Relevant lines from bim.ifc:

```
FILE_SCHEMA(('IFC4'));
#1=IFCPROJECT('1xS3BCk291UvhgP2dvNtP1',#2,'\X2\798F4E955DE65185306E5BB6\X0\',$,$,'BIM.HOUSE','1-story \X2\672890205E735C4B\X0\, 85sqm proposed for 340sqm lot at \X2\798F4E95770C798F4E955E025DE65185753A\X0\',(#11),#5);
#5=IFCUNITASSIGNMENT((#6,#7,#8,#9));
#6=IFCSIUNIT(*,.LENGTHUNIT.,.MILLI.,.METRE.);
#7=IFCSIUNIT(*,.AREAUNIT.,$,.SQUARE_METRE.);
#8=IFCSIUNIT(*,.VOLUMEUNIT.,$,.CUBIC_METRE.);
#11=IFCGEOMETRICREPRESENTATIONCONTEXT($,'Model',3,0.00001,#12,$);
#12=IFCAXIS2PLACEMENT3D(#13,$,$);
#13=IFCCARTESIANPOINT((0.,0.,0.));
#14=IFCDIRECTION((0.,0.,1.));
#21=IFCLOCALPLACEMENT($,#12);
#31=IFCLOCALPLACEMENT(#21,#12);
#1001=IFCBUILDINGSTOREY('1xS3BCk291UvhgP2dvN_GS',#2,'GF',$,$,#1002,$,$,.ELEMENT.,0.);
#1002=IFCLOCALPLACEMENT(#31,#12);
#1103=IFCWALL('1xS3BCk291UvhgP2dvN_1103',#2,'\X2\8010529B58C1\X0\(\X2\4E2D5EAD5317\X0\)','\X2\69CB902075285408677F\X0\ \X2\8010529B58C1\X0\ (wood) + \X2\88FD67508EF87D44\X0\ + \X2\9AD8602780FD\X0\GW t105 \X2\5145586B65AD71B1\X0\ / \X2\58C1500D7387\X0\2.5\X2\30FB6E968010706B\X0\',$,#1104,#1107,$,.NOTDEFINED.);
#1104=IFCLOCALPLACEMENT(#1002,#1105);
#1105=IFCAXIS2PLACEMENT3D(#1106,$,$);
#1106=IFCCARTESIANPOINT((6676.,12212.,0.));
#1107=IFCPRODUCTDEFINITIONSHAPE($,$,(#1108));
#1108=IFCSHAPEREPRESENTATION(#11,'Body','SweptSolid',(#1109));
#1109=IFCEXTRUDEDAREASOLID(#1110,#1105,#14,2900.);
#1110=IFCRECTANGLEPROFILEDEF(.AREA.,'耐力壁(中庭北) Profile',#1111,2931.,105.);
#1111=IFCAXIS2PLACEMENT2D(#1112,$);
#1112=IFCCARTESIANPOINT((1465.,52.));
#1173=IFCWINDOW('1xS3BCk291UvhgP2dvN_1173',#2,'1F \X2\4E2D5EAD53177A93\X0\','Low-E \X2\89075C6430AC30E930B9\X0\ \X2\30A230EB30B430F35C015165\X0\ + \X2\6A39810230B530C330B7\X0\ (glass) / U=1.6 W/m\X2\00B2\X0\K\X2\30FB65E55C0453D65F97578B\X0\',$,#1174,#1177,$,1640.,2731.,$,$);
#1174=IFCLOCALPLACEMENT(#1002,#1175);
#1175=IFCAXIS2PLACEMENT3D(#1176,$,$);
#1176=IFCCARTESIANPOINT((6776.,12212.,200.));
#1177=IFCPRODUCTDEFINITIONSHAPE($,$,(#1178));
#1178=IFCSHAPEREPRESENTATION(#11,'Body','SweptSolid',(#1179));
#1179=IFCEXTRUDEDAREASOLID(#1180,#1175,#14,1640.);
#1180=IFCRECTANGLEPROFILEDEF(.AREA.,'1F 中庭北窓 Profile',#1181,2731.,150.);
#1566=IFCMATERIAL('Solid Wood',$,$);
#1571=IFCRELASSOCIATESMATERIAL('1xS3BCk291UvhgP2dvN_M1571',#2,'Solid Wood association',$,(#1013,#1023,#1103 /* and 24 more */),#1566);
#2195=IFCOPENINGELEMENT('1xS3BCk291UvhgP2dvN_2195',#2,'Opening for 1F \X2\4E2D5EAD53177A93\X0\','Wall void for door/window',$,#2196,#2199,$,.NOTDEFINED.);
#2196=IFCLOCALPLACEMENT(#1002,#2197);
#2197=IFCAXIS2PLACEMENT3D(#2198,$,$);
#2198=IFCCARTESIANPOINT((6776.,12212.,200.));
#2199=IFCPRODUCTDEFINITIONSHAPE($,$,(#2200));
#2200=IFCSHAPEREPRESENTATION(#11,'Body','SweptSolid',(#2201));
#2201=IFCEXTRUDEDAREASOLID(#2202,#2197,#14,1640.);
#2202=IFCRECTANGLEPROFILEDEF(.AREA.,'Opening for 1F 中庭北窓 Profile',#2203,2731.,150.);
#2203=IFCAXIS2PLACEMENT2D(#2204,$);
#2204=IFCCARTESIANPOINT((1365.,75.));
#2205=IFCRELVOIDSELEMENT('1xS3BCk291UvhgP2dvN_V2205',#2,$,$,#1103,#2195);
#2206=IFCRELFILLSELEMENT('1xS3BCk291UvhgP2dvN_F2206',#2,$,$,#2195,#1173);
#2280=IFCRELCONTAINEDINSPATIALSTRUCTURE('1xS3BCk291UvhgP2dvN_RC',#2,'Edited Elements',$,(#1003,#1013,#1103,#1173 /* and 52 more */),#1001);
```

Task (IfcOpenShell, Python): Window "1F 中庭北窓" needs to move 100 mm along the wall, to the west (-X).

```python
import ifcopenshell
import ifcopenshell.api.geometry
import ifcopenshell.util.placement
import ifcopenshell.util.unit

model = ifcopenshell.open("bim.ifc")
unit_scale = ifcopenshell.util.unit.calculate_unit_scale(model)

window = model.by_guid("1xS3BCk291UvhgP2dvN_1173")
opening = window.FillsVoids[0].RelatingOpeningElement
wall = opening.VoidsElements[0].RelatingBuildingElement

wall_matrix = ifcopenshell.util.placement.get_local_placement(wall.ObjectPlacement)
shift = wall_matrix[:3, 0] * -0.1 / unit_scale
before = ifcopenshell.util.placement.get_local_placement(window.ObjectPlacement)[:3, 3].copy()

# The window is not placed relative to its opening, so move both.
for product in (opening, window):
    matrix = ifcopenshell.util.placement.get_local_placement(product.ObjectPlacement)
    matrix[:3, 3] += shift
    ifcopenshell.api.geometry.edit_object_placement(model, product=product, matrix=matrix, is_si=False)

after = ifcopenshell.util.placement.get_local_placement(window.ObjectPlacement)[:3, 3]
print("window moved by", (after - before).round(3) + 0.0)

model.write("bim_edited.ifc")
```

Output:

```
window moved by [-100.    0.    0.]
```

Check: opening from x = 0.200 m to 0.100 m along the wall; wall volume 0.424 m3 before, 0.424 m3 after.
